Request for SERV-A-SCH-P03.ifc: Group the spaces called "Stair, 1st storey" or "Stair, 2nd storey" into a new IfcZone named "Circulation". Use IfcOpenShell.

First a look at what the model holds.

```python
import ifcopenshell

model = ifcopenshell.open("SERV-A-SCH-P03.ifc")
print(model.schema)
seen = {}
for space in model.by_type("IfcSpace"):
    seen[space.LongName] = seen.get(space.LongName, 0) + 1
for name, count in sorted(seen.items(), key=str):
    print(count, "x", name)
print("zones:", [z.Name for z in model.by_type("IfcZone")][:20])
```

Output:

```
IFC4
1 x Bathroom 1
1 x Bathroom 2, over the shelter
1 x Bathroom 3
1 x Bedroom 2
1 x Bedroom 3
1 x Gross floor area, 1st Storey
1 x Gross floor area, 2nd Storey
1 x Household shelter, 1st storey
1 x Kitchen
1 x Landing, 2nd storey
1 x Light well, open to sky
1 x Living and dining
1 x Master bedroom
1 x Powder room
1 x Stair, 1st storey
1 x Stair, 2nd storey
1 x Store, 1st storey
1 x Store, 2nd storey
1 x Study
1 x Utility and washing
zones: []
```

```python
import ifcopenshell
import ifcopenshell.api.group
import ifcopenshell.api.root

model = ifcopenshell.open("SERV-A-SCH-P03.ifc")

names = {"Stair, 1st storey", "Stair, 2nd storey"}
spaces = [s for s in model.by_type("IfcSpace") if s.LongName in names]

zone = ifcopenshell.api.root.create_entity(model, ifc_class="IfcZone", name="Circulation")
ifcopenshell.api.group.assign_group(model, products=spaces, group=zone)
print(len(spaces), "spaces in", zone.Name)

model.write("SERV-A-SCH-P03-out.ifc")
```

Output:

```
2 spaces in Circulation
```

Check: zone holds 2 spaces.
